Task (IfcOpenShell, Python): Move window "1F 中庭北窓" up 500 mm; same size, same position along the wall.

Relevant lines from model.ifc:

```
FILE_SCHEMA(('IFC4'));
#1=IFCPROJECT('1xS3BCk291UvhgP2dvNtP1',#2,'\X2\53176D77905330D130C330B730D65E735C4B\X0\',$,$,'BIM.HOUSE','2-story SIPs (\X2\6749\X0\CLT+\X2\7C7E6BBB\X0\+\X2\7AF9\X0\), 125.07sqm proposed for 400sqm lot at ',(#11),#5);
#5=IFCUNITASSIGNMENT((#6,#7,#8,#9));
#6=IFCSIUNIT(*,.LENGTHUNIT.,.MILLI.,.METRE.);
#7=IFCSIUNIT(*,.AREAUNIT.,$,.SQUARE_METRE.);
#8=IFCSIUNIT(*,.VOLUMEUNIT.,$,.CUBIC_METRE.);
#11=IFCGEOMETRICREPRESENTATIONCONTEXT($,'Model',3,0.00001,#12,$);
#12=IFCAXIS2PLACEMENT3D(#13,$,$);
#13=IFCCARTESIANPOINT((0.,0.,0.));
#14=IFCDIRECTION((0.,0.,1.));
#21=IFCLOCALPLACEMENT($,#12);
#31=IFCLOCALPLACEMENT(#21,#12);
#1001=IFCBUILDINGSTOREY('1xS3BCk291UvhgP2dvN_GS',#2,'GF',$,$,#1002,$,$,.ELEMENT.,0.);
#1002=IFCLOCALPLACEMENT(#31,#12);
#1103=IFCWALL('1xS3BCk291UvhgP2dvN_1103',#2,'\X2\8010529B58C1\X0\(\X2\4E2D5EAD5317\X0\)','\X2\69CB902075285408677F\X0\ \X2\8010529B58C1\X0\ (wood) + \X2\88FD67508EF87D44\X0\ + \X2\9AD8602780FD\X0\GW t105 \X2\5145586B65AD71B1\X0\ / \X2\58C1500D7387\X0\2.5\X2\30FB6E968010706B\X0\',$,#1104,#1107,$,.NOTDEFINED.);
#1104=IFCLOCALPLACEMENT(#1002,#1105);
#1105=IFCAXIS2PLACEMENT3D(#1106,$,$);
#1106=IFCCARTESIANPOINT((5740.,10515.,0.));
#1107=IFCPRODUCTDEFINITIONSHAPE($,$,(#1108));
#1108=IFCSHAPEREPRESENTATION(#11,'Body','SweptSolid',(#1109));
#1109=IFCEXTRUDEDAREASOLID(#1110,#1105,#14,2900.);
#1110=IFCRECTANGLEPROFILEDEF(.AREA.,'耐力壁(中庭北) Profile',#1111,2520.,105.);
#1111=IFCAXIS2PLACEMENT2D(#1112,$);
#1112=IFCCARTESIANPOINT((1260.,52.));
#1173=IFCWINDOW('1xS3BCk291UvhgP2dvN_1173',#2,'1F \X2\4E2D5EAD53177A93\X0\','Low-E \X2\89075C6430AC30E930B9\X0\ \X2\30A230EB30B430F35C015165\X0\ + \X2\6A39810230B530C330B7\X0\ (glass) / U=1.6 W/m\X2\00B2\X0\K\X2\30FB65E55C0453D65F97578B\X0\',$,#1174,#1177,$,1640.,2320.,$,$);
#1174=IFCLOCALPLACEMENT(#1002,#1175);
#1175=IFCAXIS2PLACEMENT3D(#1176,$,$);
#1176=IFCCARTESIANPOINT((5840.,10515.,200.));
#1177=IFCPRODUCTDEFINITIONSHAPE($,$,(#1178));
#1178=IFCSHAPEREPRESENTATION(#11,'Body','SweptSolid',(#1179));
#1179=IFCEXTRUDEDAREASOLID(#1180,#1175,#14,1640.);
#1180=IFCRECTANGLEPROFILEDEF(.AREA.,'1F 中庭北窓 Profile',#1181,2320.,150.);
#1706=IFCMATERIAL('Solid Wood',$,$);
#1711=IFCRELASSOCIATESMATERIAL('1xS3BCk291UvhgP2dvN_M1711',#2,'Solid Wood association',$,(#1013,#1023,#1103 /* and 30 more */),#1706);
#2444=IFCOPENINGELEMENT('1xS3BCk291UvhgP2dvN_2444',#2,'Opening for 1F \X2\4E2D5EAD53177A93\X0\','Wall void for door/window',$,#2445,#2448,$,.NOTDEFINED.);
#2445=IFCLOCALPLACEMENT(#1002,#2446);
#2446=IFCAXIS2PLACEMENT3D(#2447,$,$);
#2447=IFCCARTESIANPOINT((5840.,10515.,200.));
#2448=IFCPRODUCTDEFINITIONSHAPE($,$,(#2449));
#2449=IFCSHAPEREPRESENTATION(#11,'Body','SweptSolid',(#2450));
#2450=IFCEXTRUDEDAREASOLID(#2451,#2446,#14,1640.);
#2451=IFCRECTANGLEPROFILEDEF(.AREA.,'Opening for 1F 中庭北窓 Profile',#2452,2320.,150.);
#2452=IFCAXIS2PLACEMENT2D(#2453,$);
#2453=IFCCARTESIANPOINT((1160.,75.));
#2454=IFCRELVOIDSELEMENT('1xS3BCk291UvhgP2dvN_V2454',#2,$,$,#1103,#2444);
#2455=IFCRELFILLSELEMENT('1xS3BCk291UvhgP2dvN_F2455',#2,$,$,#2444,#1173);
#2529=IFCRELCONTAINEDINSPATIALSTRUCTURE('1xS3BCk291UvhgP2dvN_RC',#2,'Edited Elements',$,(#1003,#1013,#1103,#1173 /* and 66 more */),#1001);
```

```python
import numpy as np
import ifcopenshell
import ifcopenshell.api.geometry
import ifcopenshell.util.placement
import ifcopenshell.util.unit

model = ifcopenshell.open("model.ifc")
unit_scale = ifcopenshell.util.unit.calculate_unit_scale(model)

window = model.by_guid("1xS3BCk291UvhgP2dvN_1173")
opening = window.FillsVoids[0].RelatingOpeningElement
dz = 0.5 / unit_scale

shift = np.array([0.0, 0.0, dz])
# The window is not placed relative to its opening, so move both.
for product in (opening, window):
    matrix = ifcopenshell.util.placement.get_local_placement(product.ObjectPlacement)
    matrix[:3, 3] += shift
    ifcopenshell.api.geometry.edit_object_placement(model, product=product, matrix=matrix, is_si=False)

print(f"moved by {dz * unit_scale:+.3f} m")

model.write("model_edited.ifc")
```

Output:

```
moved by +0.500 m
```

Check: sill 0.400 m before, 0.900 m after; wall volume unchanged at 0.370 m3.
